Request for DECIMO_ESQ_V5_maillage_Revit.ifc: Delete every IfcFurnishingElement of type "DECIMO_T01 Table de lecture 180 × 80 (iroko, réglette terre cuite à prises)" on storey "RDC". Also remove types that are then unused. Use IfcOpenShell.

First a look at what the model holds.

```python
import ifcopenshell
import ifcopenshell.util.element

model = ifcopenshell.open("DECIMO_ESQ_V5_maillage_Revit.ifc")
print(model.schema)
storey = next(s for s in model.by_type("IfcBuildingStorey") if s.Name == "RDC")
furniture = [e for e in ifcopenshell.util.element.get_decomposition(storey) if e.is_a("IfcFurnishingElement")]
seen = {}
for e in furniture:
    element_type = ifcopenshell.util.element.get_type(e)
    name = element_type.Name if element_type not in (None, e) else None
    seen[name] = seen.get(name, 0) + 1
for name, count in sorted(seen.items(), key=str):
    print(count, "x", name)
```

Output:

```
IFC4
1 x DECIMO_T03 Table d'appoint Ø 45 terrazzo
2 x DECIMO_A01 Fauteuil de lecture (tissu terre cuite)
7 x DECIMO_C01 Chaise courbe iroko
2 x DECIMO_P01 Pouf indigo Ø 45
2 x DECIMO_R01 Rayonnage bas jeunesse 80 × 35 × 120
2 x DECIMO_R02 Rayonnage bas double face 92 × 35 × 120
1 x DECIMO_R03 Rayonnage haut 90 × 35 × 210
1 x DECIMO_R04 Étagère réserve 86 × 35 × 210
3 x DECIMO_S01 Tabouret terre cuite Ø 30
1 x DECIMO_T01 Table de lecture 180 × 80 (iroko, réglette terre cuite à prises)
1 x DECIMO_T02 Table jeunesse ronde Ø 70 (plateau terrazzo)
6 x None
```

```python
import ifcopenshell
import ifcopenshell.api.root
import ifcopenshell.util.element

model = ifcopenshell.open("DECIMO_ESQ_V5_maillage_Revit.ifc")

storey = next(s for s in model.by_type("IfcBuildingStorey") if s.Name == "RDC")
furniture = [e for e in ifcopenshell.util.element.get_decomposition(storey) if e.is_a("IfcFurnishingElement")]
targets = [e for e in furniture if (t := ifcopenshell.util.element.get_type(e)) not in (None, e) and t.Name == "DECIMO_T01 Table de lecture 180 × 80 (iroko, réglette terre cuite à prises)"]
types = {ifcopenshell.util.element.get_type(e) for e in targets} - {None, *targets}

for e in targets:
    ifcopenshell.api.root.remove_product(model, product=e)
print(len(targets), "removed")

unused = [t for t in types if not ifcopenshell.util.element.get_types(t)]
for t in unused:
    ifcopenshell.api.root.remove_product(model, product=t)
print(len(unused), "unused types removed")

model.write("DECIMO_ESQ_V5_maillage_Revit_rev.ifc")
```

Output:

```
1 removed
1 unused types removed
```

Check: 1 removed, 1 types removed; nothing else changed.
